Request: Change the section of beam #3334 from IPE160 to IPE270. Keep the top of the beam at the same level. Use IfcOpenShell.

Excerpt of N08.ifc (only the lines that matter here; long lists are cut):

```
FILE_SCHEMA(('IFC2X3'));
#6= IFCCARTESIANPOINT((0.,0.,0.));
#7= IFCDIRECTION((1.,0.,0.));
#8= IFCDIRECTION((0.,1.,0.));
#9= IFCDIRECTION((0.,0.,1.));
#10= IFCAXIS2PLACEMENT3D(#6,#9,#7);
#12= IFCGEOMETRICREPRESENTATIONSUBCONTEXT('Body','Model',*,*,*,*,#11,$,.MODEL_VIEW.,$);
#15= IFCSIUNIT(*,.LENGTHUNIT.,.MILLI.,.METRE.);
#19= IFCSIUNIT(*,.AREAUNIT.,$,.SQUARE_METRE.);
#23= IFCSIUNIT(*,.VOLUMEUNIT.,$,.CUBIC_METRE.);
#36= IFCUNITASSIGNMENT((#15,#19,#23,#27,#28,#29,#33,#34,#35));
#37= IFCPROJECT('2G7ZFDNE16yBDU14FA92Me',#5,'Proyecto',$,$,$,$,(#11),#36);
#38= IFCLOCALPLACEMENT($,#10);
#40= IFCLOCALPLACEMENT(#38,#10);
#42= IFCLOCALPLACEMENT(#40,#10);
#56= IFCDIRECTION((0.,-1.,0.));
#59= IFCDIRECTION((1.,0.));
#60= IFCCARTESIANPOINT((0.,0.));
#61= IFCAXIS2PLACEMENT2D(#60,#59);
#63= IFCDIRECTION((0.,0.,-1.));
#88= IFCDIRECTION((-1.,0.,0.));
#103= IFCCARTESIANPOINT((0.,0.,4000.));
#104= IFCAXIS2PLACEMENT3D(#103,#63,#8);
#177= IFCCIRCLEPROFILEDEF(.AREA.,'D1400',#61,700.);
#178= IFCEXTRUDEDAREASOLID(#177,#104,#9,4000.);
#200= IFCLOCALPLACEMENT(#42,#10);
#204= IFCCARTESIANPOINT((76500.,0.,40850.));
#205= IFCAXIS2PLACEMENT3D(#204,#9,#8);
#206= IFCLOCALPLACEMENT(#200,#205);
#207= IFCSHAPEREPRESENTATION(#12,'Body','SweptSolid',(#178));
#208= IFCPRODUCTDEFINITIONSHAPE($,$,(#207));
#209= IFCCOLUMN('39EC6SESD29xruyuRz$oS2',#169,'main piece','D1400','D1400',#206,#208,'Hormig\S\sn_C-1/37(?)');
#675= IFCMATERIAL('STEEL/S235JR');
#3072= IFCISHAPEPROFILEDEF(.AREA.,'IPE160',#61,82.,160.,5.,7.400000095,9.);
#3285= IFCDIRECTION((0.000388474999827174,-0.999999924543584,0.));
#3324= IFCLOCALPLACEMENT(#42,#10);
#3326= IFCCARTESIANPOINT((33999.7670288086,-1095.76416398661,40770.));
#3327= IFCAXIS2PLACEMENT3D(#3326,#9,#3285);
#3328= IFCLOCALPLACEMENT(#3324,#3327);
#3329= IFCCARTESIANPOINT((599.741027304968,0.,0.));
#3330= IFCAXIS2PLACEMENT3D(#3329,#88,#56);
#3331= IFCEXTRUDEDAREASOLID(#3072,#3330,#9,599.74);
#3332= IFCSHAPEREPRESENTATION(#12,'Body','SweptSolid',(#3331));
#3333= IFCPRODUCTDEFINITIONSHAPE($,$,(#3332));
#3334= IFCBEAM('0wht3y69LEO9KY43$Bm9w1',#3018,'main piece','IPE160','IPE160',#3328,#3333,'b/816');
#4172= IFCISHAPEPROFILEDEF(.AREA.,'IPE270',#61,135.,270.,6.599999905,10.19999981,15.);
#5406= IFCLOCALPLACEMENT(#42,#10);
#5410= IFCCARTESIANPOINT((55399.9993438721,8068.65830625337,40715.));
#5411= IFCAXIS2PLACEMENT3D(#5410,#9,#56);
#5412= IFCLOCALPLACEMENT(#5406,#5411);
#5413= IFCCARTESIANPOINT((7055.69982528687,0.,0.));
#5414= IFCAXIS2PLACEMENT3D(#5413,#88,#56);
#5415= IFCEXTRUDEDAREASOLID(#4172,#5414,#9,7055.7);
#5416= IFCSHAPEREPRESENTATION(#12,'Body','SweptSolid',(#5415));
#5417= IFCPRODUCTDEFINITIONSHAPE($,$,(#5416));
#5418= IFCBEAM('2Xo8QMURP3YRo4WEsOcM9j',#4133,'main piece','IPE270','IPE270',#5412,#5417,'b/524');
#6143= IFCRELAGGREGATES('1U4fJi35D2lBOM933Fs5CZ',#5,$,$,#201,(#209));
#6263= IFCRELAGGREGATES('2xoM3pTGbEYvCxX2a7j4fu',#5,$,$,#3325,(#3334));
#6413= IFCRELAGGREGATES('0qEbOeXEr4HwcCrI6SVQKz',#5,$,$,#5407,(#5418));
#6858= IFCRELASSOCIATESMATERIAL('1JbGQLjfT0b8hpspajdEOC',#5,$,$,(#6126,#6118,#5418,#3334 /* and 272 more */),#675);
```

```python
import ifcopenshell
import ifcopenshell.util.element
import ifcopenshell.util.representation

model = ifcopenshell.open("N08.ifc")

member = model.by_guid("0wht3y69LEO9KY43$Bm9w1")
source = next(p for p in model.by_type("IfcIShapeProfileDef") if p.ProfileName == "IPE270")

body = ifcopenshell.util.representation.get_representation(member, "Model", "Body")
solid = body.Items[0]
old_profile = solid.SweptArea

# Copy the section's sizes but keep this member's own profile position.
profile = ifcopenshell.util.element.copy(model, source)
# Profiles are centred, so shift by half the change in depth to hold the top.
shift = (old_profile.OverallDepth - profile.OverallDepth) / 2
x, y = old_profile.Position.Location.Coordinates
up = (0.0, 1.0)  # upwards, in the solid's own plane
location = model.createIfcCartesianPoint((x + up[0] * shift, y + up[1] * shift))
profile.Position = model.createIfcAxis2Placement2D(location, old_profile.Position.RefDirection)
solid.SweptArea = profile
if not model.get_total_inverses(old_profile):
    ifcopenshell.util.element.remove_deep2(model, old_profile)
member.Description = member.Description.replace("IPE160", "IPE270")
member.ObjectType = member.ObjectType.replace("IPE160", "IPE270")

print(solid.SweptArea)

model.write("N08-out.ifc")
```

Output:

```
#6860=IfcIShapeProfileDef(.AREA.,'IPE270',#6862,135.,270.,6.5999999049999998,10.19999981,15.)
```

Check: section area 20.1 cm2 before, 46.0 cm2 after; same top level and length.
